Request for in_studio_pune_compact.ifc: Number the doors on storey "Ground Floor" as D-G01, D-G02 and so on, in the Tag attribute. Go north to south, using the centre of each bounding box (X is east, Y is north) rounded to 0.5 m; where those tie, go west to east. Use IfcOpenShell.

First a look at what the model holds.

```python
import ifcopenshell
import ifcopenshell.util.element
import ifcopenshell.util.placement

model = ifcopenshell.open("in_studio_pune_compact.ifc")
print(model.schema)
storey = next(s for s in model.by_type("IfcBuildingStorey") if s.Name == "Ground Floor")
doors = [e for e in ifcopenshell.util.element.get_decomposition(storey) if e.is_a("IfcDoor")]
for e in sorted(doors, key=lambda e: e.id()):
    origin = ifcopenshell.util.placement.get_local_placement(e.ObjectPlacement)[:3, 3]
    print(e.id(), e.Tag, e.Name, origin.round(2) + 0.0, sep=" | ")
```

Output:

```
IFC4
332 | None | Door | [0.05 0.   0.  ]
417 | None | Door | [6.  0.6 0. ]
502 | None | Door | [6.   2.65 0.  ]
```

```python
import ifcopenshell
import ifcopenshell.geom
import ifcopenshell.util.element
import ifcopenshell.util.shape

model = ifcopenshell.open("in_studio_pune_compact.ifc")
settings = ifcopenshell.geom.settings()
settings.set("use-world-coords", True)


def centre(element):
    shape = ifcopenshell.geom.create_shape(settings, element)
    return ifcopenshell.util.shape.get_bbox_centroid(shape.geometry)


storey = next(s for s in model.by_type("IfcBuildingStorey") if s.Name == "Ground Floor")
doors = [e for e in ifcopenshell.util.element.get_decomposition(storey) if e.is_a("IfcDoor")]

# Insertion points can sit at a corner or the storey origin, so sort by the geometry (in metres).
centres = {e: centre(e) for e in doors}
doors.sort(key=lambda e: (-round(centres[e][1] / 0.5), centres[e][0]))

for i, e in enumerate(doors, start=1):
    number = f"D-G{i:02d}"
    e.Tag = number
    print(e.id(), number)

model.write("in_studio_pune_compact-out.ifc")
```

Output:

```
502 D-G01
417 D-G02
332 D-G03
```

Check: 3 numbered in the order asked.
